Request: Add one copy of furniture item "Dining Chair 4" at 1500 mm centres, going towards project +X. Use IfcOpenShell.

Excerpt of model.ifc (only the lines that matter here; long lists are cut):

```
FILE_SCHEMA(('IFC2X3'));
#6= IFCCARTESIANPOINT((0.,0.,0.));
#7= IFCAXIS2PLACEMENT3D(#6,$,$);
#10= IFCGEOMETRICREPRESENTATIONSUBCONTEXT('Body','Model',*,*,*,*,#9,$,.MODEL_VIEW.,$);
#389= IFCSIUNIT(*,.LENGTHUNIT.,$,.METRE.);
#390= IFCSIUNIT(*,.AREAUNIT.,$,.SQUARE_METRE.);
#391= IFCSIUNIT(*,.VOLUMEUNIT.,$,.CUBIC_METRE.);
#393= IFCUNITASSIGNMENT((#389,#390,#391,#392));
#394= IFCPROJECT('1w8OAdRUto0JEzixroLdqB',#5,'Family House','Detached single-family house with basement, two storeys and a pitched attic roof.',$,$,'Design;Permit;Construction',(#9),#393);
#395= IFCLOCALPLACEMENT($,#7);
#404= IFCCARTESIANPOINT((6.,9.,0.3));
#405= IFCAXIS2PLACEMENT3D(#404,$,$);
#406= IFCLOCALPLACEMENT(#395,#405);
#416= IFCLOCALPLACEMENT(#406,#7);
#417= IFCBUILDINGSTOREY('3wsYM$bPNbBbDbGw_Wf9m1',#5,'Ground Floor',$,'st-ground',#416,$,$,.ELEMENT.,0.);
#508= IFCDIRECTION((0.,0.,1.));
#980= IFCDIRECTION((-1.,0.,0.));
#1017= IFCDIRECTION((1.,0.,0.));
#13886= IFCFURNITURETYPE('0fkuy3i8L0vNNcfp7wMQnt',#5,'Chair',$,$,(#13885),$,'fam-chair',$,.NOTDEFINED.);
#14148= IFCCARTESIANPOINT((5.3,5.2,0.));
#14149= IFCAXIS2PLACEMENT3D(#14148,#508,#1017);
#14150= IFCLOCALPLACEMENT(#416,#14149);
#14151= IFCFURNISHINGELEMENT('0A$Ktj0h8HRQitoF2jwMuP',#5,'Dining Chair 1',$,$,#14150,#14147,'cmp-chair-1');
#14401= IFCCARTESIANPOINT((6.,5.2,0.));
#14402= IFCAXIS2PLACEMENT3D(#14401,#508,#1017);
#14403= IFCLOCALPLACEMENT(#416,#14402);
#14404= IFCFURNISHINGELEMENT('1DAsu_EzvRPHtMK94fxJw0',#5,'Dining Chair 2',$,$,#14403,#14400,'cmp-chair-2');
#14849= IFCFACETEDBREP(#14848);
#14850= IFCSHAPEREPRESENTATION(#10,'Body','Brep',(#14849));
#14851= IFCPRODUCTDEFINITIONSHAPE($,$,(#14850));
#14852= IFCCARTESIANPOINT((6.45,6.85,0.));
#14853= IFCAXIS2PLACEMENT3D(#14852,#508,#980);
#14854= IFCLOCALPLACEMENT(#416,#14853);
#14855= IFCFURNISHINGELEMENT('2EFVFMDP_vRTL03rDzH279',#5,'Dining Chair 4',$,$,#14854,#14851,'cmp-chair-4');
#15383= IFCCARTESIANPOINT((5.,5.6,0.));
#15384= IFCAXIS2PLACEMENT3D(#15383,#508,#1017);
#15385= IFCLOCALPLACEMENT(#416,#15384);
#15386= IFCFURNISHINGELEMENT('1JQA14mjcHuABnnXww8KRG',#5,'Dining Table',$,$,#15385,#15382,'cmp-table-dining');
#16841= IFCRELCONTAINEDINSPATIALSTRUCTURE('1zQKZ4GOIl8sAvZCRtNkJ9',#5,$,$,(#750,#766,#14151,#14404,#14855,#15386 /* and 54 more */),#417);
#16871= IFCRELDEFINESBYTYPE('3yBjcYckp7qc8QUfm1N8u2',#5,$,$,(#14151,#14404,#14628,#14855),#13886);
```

```python
import numpy as np
import ifcopenshell
import ifcopenshell.api.geometry
import ifcopenshell.api.root
import ifcopenshell.util.element
import ifcopenshell.util.placement
import ifcopenshell.util.unit

model = ifcopenshell.open("model.ifc")
unit_scale = ifcopenshell.util.unit.calculate_unit_scale(model)


def reuse_history(source, copy):
    """copy_class also copies each property set's owner history, people and application; keep the originals."""
    for rel in copy.IsDefinedBy:
        if rel.is_a("IfcRelDefinesByProperties") and (history := rel.RelatingPropertyDefinition.OwnerHistory):
            rel.RelatingPropertyDefinition.OwnerHistory = source.OwnerHistory
            ifcopenshell.util.element.remove_deep2(model, history)


source = model.by_guid("2EFVFMDP_vRTL03rDzH279")
base = ifcopenshell.util.placement.get_local_placement(source.ObjectPlacement)
step = np.array([1.0, 0.0, 0.0]) * 1.5 / unit_scale

for i in range(1, 2):
    copy = ifcopenshell.api.root.copy_class(model, product=source)
    copy.Representation = ifcopenshell.util.element.copy_deep(
        model, source.Representation, exclude=["IfcGeometricRepresentationContext", "IfcRepresentationMap"]
    )
    copy.Tag = None
    reuse_history(source, copy)
    matrix = base.copy()
    matrix[:3, 3] += i * step
    print("added at", matrix[:3, 3].round(3) + 0.0)
    ifcopenshell.api.geometry.edit_object_placement(model, product=copy, matrix=matrix, is_si=False)

model.write("model-out.ifc")
```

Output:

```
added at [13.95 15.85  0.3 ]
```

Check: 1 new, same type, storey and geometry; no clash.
